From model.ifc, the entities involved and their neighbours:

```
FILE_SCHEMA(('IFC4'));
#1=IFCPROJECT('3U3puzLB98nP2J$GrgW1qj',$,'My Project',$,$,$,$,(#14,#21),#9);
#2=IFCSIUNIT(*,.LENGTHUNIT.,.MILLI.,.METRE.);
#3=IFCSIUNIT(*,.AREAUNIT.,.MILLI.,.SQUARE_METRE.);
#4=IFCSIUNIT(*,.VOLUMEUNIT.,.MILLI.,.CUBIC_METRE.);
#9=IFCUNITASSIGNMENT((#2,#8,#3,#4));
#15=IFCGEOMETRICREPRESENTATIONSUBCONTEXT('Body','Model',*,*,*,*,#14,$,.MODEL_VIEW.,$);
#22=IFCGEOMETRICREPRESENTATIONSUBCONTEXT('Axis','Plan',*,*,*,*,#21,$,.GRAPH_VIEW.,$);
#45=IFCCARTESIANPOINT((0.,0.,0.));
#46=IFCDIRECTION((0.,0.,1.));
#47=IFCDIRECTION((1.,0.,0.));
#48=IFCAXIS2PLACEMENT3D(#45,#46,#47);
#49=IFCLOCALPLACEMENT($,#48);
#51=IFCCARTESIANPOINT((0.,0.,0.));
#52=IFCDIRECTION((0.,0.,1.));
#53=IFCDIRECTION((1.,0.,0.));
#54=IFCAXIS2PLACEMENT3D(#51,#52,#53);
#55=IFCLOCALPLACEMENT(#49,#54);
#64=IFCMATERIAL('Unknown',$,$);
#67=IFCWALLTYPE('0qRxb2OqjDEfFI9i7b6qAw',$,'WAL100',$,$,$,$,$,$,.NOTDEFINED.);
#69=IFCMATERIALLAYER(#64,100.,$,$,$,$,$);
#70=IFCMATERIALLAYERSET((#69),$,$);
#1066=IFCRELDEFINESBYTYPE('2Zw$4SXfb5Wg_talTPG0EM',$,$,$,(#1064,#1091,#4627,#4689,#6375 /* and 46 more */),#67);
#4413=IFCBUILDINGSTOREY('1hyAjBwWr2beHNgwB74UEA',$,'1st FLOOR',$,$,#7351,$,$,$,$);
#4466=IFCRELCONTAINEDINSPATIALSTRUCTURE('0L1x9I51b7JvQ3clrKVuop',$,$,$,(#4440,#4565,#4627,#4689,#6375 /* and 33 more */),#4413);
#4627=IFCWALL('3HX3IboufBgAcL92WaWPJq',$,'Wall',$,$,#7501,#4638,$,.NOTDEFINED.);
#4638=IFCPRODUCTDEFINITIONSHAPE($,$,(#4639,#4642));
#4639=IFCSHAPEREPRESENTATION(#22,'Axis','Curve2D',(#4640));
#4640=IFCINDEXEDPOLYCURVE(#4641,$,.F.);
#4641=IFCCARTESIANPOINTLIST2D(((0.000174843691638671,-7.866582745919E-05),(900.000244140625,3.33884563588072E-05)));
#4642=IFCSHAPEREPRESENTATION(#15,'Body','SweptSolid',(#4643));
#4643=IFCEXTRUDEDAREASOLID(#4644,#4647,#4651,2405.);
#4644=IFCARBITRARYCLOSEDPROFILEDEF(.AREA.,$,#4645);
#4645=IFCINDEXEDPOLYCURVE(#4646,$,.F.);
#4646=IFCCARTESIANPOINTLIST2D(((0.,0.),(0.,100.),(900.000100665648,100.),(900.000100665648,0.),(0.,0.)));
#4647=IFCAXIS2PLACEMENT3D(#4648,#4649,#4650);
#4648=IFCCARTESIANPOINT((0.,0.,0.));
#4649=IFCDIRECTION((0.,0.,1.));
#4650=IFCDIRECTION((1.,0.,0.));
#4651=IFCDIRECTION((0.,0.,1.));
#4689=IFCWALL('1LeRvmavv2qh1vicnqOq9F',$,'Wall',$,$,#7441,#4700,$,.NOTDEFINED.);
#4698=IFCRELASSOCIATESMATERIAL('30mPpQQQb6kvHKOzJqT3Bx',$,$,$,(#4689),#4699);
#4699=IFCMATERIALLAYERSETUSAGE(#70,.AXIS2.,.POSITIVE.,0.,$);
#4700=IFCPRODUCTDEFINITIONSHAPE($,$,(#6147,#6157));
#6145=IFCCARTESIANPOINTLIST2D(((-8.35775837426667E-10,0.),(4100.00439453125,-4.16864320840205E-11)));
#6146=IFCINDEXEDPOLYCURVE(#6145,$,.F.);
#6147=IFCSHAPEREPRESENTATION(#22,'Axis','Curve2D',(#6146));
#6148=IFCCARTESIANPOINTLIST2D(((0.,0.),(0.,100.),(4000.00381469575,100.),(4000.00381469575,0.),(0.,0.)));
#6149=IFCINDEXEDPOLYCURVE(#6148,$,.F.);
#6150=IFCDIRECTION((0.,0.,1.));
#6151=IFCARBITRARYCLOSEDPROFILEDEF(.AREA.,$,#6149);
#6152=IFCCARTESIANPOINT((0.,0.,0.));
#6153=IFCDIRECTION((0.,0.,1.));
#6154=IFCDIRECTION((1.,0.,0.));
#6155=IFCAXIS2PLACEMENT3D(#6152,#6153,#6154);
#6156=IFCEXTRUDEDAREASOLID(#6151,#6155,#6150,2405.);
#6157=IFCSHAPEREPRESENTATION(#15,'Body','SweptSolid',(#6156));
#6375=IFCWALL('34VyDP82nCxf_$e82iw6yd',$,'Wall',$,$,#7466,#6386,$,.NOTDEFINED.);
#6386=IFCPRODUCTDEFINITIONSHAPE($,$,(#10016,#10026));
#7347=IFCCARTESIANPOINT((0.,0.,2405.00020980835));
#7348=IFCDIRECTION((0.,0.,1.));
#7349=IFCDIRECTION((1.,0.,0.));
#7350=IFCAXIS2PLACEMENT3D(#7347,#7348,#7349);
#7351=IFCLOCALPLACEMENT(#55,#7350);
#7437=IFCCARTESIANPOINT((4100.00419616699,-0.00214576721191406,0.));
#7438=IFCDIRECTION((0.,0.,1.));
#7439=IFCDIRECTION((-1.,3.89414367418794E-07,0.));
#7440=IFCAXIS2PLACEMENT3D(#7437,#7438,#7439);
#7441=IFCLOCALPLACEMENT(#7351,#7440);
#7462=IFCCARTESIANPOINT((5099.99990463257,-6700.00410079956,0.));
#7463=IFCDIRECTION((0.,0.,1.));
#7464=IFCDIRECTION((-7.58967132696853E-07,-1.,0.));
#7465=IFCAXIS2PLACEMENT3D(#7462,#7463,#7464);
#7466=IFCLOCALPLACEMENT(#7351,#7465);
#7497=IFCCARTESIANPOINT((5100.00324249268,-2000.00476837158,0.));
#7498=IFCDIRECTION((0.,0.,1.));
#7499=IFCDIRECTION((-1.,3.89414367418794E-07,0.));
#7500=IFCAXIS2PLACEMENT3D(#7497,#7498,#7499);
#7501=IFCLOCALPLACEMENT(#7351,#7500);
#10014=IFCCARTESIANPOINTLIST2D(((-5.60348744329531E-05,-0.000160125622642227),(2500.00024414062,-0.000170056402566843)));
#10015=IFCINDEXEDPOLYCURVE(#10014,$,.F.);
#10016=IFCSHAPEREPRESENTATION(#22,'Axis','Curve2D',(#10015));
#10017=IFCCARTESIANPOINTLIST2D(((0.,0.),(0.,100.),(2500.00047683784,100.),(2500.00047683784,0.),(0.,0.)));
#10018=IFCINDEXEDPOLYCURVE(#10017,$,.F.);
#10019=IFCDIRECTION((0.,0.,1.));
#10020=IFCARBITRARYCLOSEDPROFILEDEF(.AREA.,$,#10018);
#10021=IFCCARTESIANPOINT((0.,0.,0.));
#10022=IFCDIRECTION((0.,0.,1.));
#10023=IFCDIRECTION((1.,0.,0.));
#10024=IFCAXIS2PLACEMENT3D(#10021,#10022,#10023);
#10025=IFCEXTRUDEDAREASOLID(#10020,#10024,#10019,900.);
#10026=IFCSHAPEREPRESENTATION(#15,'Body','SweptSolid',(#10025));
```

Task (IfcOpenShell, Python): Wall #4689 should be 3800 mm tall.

```python
import ifcopenshell
import ifcopenshell.geom
import ifcopenshell.util.representation
import ifcopenshell.util.shape
import ifcopenshell.util.unit

model = ifcopenshell.open("model.ifc")
unit_scale = ifcopenshell.util.unit.calculate_unit_scale(model)
settings = ifcopenshell.geom.settings()


def volume(element):
    """Net volume in cubic metres, openings subtracted."""
    shape = ifcopenshell.geom.create_shape(settings, element)
    return ifcopenshell.util.shape.get_volume(shape.geometry)


wall = model.by_id(4689)
before = volume(wall)

body = ifcopenshell.util.representation.get_representation(wall, "Model", "Body")
solid = body.Items[0]
old_height = solid.Depth
solid.Depth = 3.8 / unit_scale
after = volume(wall)

print(f"height {old_height:g} -> {solid.Depth:g}, volume {before:.3f} -> {after:.3f} m3")

model.write("model-out.ifc")
```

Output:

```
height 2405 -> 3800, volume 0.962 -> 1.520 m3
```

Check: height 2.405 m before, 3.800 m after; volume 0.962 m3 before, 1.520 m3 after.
